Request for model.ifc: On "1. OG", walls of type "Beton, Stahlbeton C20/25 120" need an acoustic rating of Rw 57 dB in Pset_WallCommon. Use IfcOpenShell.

First a look at what the model holds.

```python
import ifcopenshell
import ifcopenshell.util.element

model = ifcopenshell.open("model.ifc")
print(model.schema)
storey = next(s for s in model.by_type("IfcBuildingStorey") if s.Name == "1. OG")
walls = [e for e in ifcopenshell.util.element.get_decomposition(storey) if e.is_a("IfcWall")]
seen = {}
for e in walls:
    element_type = ifcopenshell.util.element.get_type(e)
    key = (element_type.Name if element_type != e and element_type else None, ifcopenshell.util.element.get_pset(e, "Pset_WallCommon", "AcousticRating"))
    seen[key] = seen.get(key, 0) + 1
for (name, value), count in sorted(seen.items(), key=str):
    print(count, "x", name, "|", value)
```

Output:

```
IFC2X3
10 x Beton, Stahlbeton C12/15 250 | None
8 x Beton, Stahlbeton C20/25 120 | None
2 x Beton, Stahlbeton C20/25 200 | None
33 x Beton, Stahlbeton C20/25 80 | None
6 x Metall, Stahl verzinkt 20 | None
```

```python
import ifcopenshell
import ifcopenshell.api.pset
import ifcopenshell.util.element

model = ifcopenshell.open("model.ifc")

storey = next(s for s in model.by_type("IfcBuildingStorey") if s.Name == "1. OG")
walls = [e for e in ifcopenshell.util.element.get_decomposition(storey) if e.is_a("IfcWall")]

count = 0
for e in walls:
    element_type = ifcopenshell.util.element.get_type(e)
    if element_type in (None, e) or element_type.Name != "Beton, Stahlbeton C20/25 120":
        continue
    # add_pset returns the element's existing set when there is one.
    pset = ifcopenshell.api.pset.add_pset(model, product=e, name="Pset_WallCommon")
    ifcopenshell.api.pset.edit_pset(model, pset=pset, properties={"AcousticRating": "Rw 57 dB"})
    count += 1

print(count, "walls updated")

model.write("model_edited.ifc")
```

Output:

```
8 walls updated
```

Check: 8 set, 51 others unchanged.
